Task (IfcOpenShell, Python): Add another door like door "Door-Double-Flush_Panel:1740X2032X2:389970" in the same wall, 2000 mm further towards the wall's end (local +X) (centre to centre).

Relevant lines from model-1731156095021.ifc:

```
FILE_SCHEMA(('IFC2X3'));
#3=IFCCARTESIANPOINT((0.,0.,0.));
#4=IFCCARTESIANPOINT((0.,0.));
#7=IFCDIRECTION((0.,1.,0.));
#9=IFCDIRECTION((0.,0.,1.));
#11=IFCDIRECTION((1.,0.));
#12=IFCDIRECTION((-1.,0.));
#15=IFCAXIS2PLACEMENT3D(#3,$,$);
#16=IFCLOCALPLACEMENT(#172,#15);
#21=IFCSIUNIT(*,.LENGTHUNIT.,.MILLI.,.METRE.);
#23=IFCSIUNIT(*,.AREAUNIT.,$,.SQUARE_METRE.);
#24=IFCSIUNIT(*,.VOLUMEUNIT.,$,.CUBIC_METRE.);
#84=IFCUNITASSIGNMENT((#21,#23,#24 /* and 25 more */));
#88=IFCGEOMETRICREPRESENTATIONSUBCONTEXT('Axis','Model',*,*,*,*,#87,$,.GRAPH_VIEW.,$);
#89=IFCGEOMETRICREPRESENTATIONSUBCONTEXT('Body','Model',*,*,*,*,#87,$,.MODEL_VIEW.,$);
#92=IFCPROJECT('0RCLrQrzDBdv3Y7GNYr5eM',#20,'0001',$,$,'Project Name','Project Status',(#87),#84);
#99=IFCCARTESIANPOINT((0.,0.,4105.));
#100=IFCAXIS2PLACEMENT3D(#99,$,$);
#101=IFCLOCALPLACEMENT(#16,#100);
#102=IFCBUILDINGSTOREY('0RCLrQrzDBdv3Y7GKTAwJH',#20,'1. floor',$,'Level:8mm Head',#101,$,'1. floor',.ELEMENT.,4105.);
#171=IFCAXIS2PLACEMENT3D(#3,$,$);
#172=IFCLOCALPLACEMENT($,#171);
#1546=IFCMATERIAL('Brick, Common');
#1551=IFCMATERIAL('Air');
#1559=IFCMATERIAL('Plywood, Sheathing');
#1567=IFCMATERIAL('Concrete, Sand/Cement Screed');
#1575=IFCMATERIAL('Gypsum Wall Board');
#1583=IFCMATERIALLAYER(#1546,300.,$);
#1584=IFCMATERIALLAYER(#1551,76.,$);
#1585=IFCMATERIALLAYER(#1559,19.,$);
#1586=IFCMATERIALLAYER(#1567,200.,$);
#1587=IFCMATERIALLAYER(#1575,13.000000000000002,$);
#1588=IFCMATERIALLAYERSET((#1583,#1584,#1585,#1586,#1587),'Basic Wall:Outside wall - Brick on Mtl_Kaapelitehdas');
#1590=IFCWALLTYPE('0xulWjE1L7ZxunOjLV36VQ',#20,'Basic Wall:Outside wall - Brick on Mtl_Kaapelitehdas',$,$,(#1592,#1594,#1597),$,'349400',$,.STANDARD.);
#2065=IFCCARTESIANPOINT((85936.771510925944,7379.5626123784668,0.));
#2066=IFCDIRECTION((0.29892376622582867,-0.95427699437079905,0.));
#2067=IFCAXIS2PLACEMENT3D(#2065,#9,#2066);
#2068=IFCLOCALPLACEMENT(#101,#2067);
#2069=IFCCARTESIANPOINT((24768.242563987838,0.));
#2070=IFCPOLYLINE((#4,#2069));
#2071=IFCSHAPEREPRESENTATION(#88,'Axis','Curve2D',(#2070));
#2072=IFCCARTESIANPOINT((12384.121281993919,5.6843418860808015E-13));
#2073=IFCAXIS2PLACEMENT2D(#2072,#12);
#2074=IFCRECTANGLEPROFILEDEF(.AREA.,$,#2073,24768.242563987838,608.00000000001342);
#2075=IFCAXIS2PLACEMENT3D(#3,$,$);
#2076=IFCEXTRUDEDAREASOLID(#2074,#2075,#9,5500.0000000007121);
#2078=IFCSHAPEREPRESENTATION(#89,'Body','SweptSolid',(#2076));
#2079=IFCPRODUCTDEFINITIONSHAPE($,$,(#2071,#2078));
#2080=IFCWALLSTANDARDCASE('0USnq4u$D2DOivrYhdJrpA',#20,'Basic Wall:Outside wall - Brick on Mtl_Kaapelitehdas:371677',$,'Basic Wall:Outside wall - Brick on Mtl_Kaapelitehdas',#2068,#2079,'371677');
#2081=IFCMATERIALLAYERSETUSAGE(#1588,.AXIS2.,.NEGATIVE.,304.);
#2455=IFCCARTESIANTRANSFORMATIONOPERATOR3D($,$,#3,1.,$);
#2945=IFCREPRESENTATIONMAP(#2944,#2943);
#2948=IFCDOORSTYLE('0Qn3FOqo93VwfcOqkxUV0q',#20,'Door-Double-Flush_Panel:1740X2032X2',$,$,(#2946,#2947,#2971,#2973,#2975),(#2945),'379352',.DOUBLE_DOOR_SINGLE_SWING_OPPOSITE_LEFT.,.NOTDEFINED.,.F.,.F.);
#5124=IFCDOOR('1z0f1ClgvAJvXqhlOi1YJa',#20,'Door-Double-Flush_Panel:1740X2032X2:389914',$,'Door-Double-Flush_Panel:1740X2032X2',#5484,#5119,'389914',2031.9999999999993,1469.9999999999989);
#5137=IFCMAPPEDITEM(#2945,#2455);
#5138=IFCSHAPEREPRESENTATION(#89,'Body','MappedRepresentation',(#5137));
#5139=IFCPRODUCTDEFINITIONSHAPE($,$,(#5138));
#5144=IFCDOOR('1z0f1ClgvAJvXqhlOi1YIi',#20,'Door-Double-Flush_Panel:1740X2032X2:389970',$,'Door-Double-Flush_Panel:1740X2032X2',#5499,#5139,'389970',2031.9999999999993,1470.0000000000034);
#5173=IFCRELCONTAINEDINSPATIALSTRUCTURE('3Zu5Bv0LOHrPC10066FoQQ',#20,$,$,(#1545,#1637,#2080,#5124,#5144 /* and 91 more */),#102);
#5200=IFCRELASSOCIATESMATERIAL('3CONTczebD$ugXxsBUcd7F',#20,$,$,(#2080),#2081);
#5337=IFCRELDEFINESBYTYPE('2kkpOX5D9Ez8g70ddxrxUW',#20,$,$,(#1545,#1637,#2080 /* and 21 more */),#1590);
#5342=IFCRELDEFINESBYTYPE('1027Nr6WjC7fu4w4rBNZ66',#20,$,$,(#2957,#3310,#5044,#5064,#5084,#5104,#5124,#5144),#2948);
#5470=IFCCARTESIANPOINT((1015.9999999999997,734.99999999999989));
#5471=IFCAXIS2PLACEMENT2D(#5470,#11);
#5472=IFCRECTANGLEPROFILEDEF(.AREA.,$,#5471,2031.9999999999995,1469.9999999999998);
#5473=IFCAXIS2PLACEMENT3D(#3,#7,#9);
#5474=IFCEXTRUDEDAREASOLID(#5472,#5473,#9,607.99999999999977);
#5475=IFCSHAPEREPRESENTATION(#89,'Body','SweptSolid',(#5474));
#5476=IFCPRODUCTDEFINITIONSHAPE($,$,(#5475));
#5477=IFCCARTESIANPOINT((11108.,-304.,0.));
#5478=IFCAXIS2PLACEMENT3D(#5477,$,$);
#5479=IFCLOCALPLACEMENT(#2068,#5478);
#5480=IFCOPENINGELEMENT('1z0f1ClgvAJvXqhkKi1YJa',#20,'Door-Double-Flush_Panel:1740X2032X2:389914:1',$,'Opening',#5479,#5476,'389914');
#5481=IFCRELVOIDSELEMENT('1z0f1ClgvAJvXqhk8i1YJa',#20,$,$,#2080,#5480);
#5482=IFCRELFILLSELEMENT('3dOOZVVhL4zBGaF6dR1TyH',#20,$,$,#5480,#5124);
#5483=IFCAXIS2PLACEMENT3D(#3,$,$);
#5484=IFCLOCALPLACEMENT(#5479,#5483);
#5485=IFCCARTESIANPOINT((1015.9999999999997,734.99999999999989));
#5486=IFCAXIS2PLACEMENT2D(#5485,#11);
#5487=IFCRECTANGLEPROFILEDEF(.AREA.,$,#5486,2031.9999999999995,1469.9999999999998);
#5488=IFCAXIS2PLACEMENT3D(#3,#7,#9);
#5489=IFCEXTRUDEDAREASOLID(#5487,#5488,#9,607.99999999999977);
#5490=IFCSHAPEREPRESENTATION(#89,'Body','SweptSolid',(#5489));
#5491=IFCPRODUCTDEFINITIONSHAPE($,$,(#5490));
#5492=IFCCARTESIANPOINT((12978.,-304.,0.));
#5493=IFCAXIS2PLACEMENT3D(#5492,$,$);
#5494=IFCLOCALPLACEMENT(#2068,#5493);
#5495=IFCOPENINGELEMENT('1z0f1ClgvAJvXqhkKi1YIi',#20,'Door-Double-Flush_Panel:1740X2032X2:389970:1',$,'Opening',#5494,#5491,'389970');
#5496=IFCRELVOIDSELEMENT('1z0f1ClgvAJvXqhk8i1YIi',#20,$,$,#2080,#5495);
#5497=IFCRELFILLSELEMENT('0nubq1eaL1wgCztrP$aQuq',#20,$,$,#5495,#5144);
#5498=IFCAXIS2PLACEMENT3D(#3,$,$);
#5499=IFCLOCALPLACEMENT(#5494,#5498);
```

```python
import ifcopenshell
import ifcopenshell.api.feature
import ifcopenshell.api.geometry
import ifcopenshell.api.root
import ifcopenshell.geom
import ifcopenshell.util.element
import ifcopenshell.util.placement
import ifcopenshell.util.shape
import ifcopenshell.util.unit

model = ifcopenshell.open("model-1731156095021.ifc")
unit_scale = ifcopenshell.util.unit.calculate_unit_scale(model)
settings = ifcopenshell.geom.settings()


def volume(element):
    """Net volume in cubic metres, openings subtracted."""
    shape = ifcopenshell.geom.create_shape(settings, element)
    return ifcopenshell.util.shape.get_volume(shape.geometry)


def reuse_history(source, copy):
    """copy_class also copies each property set's owner history, people and application; keep the originals."""
    for rel in copy.IsDefinedBy:
        if rel.is_a("IfcRelDefinesByProperties") and (history := rel.RelatingPropertyDefinition.OwnerHistory):
            rel.RelatingPropertyDefinition.OwnerHistory = source.OwnerHistory
            ifcopenshell.util.element.remove_deep2(model, history)


door = model.by_guid("1z0f1ClgvAJvXqhlOi1YIi")
opening = door.FillsVoids[0].RelatingOpeningElement
wall = opening.VoidsElements[0].RelatingBuildingElement
before = volume(wall)
shift = ifcopenshell.util.placement.get_local_placement(wall.ObjectPlacement)[:3, 0] * 2 / unit_scale

# copy_class copies the void relationship, type, container and properties, but no geometry.
new_opening = ifcopenshell.api.root.copy_class(model, product=opening)
new_opening.Representation = ifcopenshell.util.element.copy_deep(
    model, opening.Representation, exclude=["IfcGeometricRepresentationContext", "IfcRepresentationMap"]
)
new_opening.Name = "Door-Double-Flush_Panel:1740X2032X2"
new_opening.Tag = None
new_door = ifcopenshell.api.root.copy_class(model, product=door)
new_door.Representation = ifcopenshell.util.element.copy_deep(
    model, door.Representation, exclude=["IfcGeometricRepresentationContext", "IfcRepresentationMap"]
)
new_door.Name = "Door-Double-Flush_Panel:1740X2032X2"
new_door.Tag = None
reuse_history(door, new_door)
fills = ifcopenshell.api.feature.add_filling(model, opening=new_opening, element=new_door)
fills.OwnerHistory = new_door.OwnerHistory  # required in IFC2X3

for old, new in ((opening, new_opening), (door, new_door)):
    matrix = ifcopenshell.util.placement.get_local_placement(old.ObjectPlacement)
    matrix[:3, 3] += shift
    ifcopenshell.api.geometry.edit_object_placement(model, product=new, matrix=matrix, is_si=False)

after = volume(wall)

print(f"wall volume {before:.3f} -> {after:.3f} m3")

model.write("model-1731156095021_rev.ifc")
```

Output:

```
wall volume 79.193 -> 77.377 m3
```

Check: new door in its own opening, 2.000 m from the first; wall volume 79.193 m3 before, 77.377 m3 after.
